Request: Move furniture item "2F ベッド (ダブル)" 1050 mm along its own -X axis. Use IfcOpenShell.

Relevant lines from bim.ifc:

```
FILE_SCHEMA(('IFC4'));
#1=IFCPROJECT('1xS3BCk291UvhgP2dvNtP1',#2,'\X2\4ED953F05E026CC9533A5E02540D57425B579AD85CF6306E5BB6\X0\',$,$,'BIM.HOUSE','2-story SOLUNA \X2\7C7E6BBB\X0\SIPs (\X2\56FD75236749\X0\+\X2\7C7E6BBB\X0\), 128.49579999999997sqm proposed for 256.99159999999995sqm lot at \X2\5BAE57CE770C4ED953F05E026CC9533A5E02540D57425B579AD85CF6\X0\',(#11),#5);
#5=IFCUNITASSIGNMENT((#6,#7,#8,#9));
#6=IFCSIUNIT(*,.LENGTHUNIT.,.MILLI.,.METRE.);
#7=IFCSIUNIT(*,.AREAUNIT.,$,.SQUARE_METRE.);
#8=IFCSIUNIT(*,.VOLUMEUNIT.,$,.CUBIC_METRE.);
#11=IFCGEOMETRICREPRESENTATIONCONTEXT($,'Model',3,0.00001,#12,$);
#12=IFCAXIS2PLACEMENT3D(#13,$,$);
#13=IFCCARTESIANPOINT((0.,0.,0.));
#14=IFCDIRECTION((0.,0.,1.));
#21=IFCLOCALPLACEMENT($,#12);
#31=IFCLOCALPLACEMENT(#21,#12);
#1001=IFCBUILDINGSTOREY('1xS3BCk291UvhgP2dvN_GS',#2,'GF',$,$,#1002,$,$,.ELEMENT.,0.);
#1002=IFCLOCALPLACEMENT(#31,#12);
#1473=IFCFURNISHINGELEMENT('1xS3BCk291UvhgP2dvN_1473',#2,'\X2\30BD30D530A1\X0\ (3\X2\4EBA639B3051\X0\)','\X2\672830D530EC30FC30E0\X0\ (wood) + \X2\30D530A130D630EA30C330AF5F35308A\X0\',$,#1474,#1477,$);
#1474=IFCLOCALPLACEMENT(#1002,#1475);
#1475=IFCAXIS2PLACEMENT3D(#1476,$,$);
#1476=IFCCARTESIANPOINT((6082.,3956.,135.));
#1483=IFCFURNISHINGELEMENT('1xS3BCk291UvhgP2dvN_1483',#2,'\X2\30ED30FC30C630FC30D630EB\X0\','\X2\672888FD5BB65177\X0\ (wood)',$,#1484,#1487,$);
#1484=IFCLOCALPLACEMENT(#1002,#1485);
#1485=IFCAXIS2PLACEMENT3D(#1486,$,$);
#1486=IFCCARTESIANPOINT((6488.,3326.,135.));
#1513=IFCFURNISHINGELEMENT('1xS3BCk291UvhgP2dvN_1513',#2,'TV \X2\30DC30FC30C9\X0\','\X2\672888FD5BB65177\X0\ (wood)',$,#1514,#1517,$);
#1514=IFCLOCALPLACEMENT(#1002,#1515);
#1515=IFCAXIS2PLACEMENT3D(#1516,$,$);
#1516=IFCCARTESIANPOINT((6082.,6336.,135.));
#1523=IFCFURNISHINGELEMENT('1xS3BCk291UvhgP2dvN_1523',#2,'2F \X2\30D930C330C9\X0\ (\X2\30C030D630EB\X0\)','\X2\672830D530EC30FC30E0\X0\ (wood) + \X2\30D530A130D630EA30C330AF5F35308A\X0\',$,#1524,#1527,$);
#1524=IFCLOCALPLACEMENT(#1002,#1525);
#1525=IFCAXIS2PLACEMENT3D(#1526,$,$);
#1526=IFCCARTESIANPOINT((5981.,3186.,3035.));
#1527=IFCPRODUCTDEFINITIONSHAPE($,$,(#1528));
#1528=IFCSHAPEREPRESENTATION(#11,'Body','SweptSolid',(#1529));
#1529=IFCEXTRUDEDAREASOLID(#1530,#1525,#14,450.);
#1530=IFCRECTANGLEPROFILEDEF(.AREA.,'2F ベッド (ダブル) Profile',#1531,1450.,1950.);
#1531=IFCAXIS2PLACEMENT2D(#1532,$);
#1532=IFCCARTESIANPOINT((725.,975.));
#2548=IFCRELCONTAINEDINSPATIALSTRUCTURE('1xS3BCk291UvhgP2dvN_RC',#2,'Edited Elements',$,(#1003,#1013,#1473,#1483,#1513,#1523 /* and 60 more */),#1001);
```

```python
import ifcopenshell
import ifcopenshell.api.geometry
import ifcopenshell.util.placement

model = ifcopenshell.open("bim.ifc")

item = model.by_guid("1xS3BCk291UvhgP2dvN_1523")
matrix = ifcopenshell.util.placement.get_local_placement(item.ObjectPlacement)
matrix[:3, 3] -= matrix[:3, 0] * 1050.0
ifcopenshell.api.geometry.edit_object_placement(model, product=item, matrix=matrix, is_si=False)

print(ifcopenshell.util.placement.get_local_placement(item.ObjectPlacement).round(3) + 0.0)

model.write("bim_v2.ifc")
```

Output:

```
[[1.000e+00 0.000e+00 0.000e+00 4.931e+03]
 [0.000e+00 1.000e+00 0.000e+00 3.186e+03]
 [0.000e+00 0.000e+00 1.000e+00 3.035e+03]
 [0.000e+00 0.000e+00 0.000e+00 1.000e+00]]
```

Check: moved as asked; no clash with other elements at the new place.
